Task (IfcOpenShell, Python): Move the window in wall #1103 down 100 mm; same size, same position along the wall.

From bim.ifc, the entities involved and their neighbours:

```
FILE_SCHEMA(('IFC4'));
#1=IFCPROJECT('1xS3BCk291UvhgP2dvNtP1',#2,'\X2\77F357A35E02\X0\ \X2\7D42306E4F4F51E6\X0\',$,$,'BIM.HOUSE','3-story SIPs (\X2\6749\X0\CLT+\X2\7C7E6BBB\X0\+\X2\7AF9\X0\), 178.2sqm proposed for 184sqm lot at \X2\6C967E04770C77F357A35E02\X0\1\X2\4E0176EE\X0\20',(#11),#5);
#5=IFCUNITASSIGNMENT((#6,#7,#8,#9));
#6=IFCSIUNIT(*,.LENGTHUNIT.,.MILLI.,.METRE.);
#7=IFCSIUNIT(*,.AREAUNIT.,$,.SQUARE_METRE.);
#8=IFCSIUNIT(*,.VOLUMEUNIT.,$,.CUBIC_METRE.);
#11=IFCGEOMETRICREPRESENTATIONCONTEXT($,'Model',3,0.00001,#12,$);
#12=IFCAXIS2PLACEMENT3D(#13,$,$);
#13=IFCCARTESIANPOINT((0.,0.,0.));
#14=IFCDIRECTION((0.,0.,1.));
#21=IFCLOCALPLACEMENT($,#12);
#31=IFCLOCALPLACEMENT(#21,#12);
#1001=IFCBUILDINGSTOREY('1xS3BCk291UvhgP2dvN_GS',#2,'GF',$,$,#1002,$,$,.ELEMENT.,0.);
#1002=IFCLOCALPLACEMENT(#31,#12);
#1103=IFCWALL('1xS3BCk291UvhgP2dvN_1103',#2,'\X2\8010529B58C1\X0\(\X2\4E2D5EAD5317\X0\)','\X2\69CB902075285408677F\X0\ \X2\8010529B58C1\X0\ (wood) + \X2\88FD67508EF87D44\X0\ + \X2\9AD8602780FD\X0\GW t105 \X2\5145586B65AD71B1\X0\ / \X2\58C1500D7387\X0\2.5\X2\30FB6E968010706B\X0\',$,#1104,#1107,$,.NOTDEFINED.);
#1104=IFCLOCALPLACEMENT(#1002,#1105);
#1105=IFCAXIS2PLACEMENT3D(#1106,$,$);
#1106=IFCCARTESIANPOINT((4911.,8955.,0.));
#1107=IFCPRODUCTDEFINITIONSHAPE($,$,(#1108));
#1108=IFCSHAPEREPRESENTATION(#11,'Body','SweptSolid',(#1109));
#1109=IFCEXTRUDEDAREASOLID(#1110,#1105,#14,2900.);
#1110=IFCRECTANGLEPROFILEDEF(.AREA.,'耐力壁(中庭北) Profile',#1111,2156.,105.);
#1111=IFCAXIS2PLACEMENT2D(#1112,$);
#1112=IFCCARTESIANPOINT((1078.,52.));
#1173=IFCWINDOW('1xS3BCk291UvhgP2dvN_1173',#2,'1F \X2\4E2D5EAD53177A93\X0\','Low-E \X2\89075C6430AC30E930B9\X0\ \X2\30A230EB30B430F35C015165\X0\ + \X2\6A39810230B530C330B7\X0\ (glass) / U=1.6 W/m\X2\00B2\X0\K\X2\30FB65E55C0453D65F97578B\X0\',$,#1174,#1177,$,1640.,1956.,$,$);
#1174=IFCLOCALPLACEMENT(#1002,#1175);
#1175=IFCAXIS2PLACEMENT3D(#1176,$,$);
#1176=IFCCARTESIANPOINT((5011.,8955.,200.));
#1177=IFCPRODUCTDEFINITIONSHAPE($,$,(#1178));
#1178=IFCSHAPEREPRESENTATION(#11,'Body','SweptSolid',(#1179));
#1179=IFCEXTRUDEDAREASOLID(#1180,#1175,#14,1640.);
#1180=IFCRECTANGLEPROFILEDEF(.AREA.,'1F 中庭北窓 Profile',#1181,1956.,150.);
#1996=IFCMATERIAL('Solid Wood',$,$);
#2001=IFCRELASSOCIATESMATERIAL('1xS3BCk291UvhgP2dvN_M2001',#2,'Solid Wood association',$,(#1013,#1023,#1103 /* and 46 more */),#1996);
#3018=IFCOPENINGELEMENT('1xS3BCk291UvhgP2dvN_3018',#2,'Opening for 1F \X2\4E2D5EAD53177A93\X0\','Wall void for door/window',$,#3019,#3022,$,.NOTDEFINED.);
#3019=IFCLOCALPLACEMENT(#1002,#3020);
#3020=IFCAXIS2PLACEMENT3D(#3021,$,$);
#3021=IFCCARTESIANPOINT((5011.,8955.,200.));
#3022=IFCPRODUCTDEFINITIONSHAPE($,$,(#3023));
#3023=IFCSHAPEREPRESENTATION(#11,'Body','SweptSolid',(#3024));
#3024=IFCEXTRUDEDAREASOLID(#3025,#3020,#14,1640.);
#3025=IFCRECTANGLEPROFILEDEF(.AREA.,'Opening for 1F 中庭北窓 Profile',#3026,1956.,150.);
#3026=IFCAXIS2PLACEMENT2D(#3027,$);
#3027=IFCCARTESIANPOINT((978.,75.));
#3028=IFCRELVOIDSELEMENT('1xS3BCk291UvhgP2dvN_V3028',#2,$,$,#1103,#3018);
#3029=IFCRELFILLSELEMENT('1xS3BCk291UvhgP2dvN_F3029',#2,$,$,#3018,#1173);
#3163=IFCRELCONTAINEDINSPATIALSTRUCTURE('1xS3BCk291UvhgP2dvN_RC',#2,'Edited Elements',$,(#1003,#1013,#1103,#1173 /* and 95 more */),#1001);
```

```python
import numpy as np
import ifcopenshell
import ifcopenshell.api.geometry
import ifcopenshell.util.placement
import ifcopenshell.util.unit

model = ifcopenshell.open("bim.ifc")
unit_scale = ifcopenshell.util.unit.calculate_unit_scale(model)

window = model.by_id(1173)
opening = window.FillsVoids[0].RelatingOpeningElement
dz = -0.1 / unit_scale

shift = np.array([0.0, 0.0, dz])
# The window is not placed relative to its opening, so move both.
for product in (opening, window):
    matrix = ifcopenshell.util.placement.get_local_placement(product.ObjectPlacement)
    matrix[:3, 3] += shift
    ifcopenshell.api.geometry.edit_object_placement(model, product=product, matrix=matrix, is_si=False)

print(f"moved by {dz * unit_scale:+.3f} m")

model.write("bim_updated.ifc")
```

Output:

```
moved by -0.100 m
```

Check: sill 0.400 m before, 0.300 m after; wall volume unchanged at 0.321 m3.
